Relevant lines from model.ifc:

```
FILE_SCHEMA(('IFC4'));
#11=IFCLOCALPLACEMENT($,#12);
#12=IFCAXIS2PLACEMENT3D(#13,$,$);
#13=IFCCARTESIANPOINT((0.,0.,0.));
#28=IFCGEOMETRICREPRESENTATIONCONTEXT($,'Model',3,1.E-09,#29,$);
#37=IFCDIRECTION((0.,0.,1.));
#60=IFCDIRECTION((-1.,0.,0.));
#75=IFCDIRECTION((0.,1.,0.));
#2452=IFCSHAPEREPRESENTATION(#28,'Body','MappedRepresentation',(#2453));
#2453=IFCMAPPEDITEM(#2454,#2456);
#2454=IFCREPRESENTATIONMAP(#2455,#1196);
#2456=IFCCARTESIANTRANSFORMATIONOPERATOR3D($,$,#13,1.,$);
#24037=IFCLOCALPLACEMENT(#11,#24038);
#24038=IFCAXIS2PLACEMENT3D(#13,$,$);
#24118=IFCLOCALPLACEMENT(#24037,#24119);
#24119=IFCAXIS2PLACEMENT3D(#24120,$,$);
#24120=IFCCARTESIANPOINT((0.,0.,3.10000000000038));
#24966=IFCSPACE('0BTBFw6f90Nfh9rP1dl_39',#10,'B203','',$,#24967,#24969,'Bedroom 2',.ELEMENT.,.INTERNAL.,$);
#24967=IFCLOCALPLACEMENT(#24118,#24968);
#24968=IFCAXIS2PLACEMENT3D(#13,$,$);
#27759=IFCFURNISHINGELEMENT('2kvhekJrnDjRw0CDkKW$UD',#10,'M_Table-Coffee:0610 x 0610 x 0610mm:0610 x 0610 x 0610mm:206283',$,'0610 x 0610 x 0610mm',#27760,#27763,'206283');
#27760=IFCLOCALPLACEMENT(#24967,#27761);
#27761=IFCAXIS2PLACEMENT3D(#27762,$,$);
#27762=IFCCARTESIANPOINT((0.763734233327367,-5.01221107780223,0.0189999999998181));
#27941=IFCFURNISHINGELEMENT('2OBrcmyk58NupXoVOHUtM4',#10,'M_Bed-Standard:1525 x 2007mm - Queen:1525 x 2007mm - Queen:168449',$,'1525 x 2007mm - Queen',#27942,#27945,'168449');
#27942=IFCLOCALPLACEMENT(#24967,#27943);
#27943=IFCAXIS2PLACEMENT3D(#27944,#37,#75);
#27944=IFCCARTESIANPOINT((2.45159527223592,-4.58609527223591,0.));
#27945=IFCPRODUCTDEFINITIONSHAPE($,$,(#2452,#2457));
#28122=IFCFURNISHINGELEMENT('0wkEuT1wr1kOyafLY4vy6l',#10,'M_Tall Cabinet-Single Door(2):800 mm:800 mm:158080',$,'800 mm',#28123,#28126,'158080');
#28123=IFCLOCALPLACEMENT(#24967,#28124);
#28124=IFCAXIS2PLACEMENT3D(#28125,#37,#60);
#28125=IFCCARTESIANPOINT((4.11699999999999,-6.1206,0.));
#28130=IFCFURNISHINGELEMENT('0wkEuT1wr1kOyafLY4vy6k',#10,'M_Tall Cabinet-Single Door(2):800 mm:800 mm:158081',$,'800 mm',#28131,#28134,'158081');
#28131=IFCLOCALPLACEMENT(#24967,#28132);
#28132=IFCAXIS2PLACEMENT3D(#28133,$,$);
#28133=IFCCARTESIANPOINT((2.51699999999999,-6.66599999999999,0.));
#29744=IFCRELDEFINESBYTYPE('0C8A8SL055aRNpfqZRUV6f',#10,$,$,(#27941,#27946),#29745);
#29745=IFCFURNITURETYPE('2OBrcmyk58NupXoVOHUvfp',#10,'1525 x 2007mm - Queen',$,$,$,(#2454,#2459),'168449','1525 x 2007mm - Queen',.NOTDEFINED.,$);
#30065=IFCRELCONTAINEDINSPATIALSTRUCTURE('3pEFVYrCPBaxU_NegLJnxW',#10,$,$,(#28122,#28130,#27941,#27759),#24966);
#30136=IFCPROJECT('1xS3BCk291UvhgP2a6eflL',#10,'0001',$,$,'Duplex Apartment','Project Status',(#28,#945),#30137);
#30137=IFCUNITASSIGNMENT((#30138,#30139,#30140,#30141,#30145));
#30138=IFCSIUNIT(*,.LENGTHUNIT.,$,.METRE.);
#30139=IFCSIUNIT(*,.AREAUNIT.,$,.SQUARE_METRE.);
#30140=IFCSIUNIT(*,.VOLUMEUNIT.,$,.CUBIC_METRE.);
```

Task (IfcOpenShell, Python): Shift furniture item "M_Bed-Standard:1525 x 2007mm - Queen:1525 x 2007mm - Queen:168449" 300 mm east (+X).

```python
import ifcopenshell
import ifcopenshell.api.geometry
import ifcopenshell.util.placement
import ifcopenshell.util.unit

model = ifcopenshell.open("model.ifc")
unit_scale = ifcopenshell.util.unit.calculate_unit_scale(model)

item = model.by_guid("2OBrcmyk58NupXoVOHUtM4")
matrix = ifcopenshell.util.placement.get_local_placement(item.ObjectPlacement)
matrix[0, 3] += 0.3 / unit_scale
ifcopenshell.api.geometry.edit_object_placement(model, product=item, matrix=matrix, is_si=False)

print(ifcopenshell.util.placement.get_local_placement(item.ObjectPlacement).round(3) + 0.0)

model.write("model-out.ifc")
```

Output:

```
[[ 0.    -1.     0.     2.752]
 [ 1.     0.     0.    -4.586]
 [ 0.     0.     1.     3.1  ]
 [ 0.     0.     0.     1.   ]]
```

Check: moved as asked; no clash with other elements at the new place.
